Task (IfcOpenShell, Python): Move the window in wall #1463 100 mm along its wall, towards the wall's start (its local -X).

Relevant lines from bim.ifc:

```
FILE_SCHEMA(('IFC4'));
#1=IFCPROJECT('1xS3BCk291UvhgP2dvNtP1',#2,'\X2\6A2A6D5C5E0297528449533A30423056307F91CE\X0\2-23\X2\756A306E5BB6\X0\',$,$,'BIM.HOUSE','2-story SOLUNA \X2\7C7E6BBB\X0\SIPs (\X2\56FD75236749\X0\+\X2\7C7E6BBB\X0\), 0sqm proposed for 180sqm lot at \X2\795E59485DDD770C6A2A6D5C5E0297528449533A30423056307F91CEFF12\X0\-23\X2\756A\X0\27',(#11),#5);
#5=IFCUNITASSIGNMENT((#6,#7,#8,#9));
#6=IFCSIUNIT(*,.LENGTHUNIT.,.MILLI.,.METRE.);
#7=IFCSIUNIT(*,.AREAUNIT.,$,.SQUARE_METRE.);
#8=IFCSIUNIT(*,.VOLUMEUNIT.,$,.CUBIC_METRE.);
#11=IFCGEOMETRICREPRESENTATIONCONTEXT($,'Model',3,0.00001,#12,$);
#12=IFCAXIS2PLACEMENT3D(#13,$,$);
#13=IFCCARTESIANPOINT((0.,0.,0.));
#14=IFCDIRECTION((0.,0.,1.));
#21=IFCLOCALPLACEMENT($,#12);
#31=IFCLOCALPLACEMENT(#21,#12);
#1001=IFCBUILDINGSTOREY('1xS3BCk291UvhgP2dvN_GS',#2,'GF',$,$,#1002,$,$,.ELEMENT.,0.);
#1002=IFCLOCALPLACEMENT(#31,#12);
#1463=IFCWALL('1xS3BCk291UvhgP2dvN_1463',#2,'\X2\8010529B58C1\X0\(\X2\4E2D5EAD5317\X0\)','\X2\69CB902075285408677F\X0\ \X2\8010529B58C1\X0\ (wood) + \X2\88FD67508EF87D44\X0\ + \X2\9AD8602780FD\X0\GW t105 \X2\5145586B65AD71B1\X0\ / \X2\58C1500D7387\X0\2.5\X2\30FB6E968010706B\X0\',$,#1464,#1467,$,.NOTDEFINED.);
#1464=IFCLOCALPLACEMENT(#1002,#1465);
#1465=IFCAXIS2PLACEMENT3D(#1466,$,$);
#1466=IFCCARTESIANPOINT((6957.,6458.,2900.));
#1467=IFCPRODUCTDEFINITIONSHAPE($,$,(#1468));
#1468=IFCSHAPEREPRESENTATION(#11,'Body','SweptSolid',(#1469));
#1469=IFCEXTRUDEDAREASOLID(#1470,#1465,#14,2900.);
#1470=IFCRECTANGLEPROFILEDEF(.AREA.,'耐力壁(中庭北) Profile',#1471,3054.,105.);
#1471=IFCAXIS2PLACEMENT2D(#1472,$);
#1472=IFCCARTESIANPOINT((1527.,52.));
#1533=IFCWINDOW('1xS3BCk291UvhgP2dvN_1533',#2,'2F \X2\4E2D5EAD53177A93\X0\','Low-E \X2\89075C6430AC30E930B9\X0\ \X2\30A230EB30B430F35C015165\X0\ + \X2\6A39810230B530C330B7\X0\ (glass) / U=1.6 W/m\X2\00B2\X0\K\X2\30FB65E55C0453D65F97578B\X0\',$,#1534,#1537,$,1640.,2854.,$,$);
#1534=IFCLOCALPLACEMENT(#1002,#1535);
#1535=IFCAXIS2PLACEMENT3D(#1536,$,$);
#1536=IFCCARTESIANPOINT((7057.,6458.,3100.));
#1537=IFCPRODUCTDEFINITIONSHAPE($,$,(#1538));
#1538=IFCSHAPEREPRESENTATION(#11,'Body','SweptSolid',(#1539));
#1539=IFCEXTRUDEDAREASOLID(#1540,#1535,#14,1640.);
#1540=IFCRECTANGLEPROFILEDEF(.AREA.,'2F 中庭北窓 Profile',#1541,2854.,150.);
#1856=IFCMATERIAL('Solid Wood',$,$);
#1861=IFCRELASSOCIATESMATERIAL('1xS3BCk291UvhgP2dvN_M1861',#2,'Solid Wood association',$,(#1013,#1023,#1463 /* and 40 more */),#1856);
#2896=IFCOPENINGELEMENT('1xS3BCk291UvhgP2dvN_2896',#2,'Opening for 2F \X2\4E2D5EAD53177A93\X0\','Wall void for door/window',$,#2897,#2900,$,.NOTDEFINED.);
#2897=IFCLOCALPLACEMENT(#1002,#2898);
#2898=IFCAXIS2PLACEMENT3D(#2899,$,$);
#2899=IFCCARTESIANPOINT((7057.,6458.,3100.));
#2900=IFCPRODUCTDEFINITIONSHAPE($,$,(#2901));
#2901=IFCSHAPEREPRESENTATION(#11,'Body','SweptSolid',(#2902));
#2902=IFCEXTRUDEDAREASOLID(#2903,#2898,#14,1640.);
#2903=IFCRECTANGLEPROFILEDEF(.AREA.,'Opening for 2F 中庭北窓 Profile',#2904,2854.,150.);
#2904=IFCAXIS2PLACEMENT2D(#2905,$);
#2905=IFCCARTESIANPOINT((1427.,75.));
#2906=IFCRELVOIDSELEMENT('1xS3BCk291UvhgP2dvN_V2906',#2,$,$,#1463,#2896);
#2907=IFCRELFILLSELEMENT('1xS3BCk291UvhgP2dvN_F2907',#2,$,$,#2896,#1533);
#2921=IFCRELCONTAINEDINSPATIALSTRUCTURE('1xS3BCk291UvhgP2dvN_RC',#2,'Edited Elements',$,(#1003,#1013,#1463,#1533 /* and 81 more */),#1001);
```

```python
import ifcopenshell
import ifcopenshell.api.geometry
import ifcopenshell.util.placement
import ifcopenshell.util.unit

model = ifcopenshell.open("bim.ifc")
unit_scale = ifcopenshell.util.unit.calculate_unit_scale(model)

window = model.by_guid("1xS3BCk291UvhgP2dvN_1533")
opening = window.FillsVoids[0].RelatingOpeningElement
wall = opening.VoidsElements[0].RelatingBuildingElement

wall_matrix = ifcopenshell.util.placement.get_local_placement(wall.ObjectPlacement)
shift = wall_matrix[:3, 0] * -0.1 / unit_scale
before = ifcopenshell.util.placement.get_local_placement(window.ObjectPlacement)[:3, 3].copy()

# The window is not placed relative to its opening, so move both.
for product in (opening, window):
    matrix = ifcopenshell.util.placement.get_local_placement(product.ObjectPlacement)
    matrix[:3, 3] += shift
    ifcopenshell.api.geometry.edit_object_placement(model, product=product, matrix=matrix, is_si=False)

after = ifcopenshell.util.placement.get_local_placement(window.ObjectPlacement)[:3, 3]
print("window moved by", (after - before).round(3) + 0.0)

model.write("bim-out.ifc")
```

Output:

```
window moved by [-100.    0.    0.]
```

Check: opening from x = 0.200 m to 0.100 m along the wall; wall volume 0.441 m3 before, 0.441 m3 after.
